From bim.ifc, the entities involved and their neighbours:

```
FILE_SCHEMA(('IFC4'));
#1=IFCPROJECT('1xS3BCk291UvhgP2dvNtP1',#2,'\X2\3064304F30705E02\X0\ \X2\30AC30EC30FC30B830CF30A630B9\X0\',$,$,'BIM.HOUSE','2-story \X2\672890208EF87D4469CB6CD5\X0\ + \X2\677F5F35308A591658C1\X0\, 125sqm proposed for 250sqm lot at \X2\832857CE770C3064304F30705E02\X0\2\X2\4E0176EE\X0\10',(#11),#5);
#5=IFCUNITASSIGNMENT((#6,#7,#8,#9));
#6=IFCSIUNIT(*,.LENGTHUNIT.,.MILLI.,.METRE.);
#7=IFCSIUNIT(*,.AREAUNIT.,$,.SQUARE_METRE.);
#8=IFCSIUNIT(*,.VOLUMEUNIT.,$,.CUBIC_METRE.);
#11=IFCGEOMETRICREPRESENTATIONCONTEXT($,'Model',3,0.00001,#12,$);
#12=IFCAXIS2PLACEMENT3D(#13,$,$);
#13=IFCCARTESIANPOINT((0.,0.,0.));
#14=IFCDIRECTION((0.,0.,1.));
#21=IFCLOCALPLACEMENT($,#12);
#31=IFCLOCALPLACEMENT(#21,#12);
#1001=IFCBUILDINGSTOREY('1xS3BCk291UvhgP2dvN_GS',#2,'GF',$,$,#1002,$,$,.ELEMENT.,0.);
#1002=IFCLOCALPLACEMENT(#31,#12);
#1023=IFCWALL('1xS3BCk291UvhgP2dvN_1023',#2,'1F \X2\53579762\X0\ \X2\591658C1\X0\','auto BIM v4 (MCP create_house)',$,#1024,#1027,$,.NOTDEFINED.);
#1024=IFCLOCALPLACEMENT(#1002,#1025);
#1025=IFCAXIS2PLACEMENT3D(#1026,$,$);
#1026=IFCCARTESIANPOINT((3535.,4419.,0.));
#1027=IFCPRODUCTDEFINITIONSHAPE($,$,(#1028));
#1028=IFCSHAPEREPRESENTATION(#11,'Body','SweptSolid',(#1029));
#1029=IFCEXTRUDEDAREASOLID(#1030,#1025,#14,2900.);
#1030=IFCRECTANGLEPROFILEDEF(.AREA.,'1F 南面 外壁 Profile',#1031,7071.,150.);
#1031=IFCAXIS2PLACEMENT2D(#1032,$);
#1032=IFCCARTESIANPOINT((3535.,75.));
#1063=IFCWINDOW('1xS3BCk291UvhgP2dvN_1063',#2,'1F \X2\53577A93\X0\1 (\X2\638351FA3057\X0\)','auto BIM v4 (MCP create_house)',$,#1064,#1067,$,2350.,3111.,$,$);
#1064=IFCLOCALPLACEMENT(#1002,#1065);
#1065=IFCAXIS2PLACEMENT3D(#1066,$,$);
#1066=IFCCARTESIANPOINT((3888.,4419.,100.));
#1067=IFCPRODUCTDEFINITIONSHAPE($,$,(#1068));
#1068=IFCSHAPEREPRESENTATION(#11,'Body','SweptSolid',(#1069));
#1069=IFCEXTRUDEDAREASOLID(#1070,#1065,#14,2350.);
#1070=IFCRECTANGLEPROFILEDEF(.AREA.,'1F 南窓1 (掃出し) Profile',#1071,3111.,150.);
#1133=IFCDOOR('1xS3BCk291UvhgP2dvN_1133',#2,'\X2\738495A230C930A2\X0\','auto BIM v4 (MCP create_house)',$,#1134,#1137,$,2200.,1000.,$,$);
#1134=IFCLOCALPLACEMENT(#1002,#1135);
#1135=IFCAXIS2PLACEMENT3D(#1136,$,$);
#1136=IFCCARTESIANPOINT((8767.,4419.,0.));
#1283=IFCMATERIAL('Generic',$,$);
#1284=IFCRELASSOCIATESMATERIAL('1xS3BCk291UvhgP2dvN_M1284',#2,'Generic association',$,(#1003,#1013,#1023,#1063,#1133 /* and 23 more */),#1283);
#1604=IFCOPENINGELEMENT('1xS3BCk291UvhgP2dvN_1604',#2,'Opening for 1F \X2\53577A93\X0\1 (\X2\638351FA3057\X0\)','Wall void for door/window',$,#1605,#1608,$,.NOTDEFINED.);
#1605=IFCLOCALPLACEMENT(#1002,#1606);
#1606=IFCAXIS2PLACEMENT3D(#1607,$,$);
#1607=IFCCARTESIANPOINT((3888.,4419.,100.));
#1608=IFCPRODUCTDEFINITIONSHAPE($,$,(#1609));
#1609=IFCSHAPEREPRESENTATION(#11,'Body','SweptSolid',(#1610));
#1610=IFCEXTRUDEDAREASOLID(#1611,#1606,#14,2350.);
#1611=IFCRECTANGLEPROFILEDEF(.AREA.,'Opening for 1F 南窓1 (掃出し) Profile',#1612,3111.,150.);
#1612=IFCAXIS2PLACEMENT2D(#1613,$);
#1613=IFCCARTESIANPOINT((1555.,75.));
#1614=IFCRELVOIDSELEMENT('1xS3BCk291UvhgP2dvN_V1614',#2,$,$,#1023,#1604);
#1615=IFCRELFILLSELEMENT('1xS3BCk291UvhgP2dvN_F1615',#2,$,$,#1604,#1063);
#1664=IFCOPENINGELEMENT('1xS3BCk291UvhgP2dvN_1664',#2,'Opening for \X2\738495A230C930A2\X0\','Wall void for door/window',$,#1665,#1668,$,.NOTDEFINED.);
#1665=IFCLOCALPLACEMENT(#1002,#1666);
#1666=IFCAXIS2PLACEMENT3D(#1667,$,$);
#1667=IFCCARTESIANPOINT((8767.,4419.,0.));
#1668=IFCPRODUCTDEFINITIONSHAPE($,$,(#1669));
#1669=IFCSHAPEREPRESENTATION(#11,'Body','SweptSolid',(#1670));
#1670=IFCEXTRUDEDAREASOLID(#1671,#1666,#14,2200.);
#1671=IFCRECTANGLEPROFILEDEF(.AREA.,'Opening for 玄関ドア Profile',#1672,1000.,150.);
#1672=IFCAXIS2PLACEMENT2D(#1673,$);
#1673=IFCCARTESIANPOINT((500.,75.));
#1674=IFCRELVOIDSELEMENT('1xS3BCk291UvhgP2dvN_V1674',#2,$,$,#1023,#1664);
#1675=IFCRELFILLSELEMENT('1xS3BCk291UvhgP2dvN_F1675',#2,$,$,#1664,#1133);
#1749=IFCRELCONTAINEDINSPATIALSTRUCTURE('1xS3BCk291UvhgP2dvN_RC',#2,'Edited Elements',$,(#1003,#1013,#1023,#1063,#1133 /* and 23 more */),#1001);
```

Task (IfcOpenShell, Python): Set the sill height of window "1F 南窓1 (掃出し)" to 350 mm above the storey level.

```python
import numpy as np
import ifcopenshell
import ifcopenshell.api.geometry
import ifcopenshell.geom
import ifcopenshell.util.element
import ifcopenshell.util.placement
import ifcopenshell.util.shape
import ifcopenshell.util.unit

model = ifcopenshell.open("bim.ifc")
unit_scale = ifcopenshell.util.unit.calculate_unit_scale(model)

window = model.by_guid("1xS3BCk291UvhgP2dvN_1063")
opening = window.FillsVoids[0].RelatingOpeningElement
storey = ifcopenshell.util.element.get_container(window, ifc_class="IfcBuildingStorey")
level = ifcopenshell.util.placement.get_local_placement(storey.ObjectPlacement)[2, 3]

# The opening's origin need not be at the sill, so measure its lowest point.
shape = ifcopenshell.geom.create_shape(ifcopenshell.geom.settings(), opening)
bottom = ifcopenshell.util.shape.get_shape_bottom_elevation(shape, shape.geometry) / unit_scale
dz = level + 350.0 - bottom

shift = np.array([0.0, 0.0, dz])
# The window is not placed relative to its opening, so move both.
for product in (opening, window):
    matrix = ifcopenshell.util.placement.get_local_placement(product.ObjectPlacement)
    matrix[:3, 3] += shift
    ifcopenshell.api.geometry.edit_object_placement(model, product=product, matrix=matrix, is_si=False)

print(f"moved by {dz * unit_scale:+.3f} m")

model.write("bim_v2.ifc")
```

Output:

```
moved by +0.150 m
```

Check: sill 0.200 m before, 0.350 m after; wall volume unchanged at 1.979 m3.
